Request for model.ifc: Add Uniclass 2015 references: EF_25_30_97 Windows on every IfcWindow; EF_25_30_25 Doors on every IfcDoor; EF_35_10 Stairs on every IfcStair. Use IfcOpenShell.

First a look at what the model holds.

```python
import ifcopenshell

model = ifcopenshell.open("model.ifc")
print(model.schema)
print("classifications:", [c.Name for c in model.by_type("IfcClassification")])
for ifc_class in ("IfcDoor", "IfcRoof", "IfcStair", "IfcWall", "IfcWindow"):
    print(ifc_class, len(model.by_type(ifc_class)))
```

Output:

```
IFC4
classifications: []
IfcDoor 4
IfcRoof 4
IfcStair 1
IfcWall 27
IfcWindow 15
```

```python
import ifcopenshell
import ifcopenshell.api.classification

model = ifcopenshell.open("model.ifc")

system = ifcopenshell.api.classification.add_classification(model, classification="Uniclass 2015")

codes = {
    "IfcWindow": ("EF_25_30_97", "Windows"),
    "IfcDoor": ("EF_25_30_25", "Doors"),
    "IfcStair": ("EF_35_10", "Stairs"),
}
for ifc_class, (code, name) in codes.items():
    products = model.by_type(ifc_class)
    ifcopenshell.api.classification.add_reference(
        model, products=products, classification=system, identification=code, name=name
    )
    print(code, len(products))

model.write("model_edited.ifc")
```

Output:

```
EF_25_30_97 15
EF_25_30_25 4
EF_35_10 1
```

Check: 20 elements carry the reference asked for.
